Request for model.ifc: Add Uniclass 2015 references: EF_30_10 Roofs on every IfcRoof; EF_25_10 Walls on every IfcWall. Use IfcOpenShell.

First a look at what the model holds.

```python
import ifcopenshell

model = ifcopenshell.open("model.ifc")
print(model.schema)
print("classifications:", [c.Name for c in model.by_type("IfcClassification")])
for ifc_class in ("IfcDoor", "IfcRoof", "IfcStair", "IfcWall", "IfcWindow"):
    print(ifc_class, len(model.by_type(ifc_class)))
```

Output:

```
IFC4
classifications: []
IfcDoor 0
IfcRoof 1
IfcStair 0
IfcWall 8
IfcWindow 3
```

```python
import ifcopenshell
import ifcopenshell.api.classification

model = ifcopenshell.open("model.ifc")

system = ifcopenshell.api.classification.add_classification(model, classification="Uniclass 2015")

codes = {
    "IfcRoof": ("EF_30_10", "Roofs"),
    "IfcWall": ("EF_25_10", "Walls"),
}
for ifc_class, (code, name) in codes.items():
    products = model.by_type(ifc_class)
    ifcopenshell.api.classification.add_reference(
        model, products=products, classification=system, identification=code, name=name
    )
    print(code, len(products))

model.write("model_updated.ifc")
```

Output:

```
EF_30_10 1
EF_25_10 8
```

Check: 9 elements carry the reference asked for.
